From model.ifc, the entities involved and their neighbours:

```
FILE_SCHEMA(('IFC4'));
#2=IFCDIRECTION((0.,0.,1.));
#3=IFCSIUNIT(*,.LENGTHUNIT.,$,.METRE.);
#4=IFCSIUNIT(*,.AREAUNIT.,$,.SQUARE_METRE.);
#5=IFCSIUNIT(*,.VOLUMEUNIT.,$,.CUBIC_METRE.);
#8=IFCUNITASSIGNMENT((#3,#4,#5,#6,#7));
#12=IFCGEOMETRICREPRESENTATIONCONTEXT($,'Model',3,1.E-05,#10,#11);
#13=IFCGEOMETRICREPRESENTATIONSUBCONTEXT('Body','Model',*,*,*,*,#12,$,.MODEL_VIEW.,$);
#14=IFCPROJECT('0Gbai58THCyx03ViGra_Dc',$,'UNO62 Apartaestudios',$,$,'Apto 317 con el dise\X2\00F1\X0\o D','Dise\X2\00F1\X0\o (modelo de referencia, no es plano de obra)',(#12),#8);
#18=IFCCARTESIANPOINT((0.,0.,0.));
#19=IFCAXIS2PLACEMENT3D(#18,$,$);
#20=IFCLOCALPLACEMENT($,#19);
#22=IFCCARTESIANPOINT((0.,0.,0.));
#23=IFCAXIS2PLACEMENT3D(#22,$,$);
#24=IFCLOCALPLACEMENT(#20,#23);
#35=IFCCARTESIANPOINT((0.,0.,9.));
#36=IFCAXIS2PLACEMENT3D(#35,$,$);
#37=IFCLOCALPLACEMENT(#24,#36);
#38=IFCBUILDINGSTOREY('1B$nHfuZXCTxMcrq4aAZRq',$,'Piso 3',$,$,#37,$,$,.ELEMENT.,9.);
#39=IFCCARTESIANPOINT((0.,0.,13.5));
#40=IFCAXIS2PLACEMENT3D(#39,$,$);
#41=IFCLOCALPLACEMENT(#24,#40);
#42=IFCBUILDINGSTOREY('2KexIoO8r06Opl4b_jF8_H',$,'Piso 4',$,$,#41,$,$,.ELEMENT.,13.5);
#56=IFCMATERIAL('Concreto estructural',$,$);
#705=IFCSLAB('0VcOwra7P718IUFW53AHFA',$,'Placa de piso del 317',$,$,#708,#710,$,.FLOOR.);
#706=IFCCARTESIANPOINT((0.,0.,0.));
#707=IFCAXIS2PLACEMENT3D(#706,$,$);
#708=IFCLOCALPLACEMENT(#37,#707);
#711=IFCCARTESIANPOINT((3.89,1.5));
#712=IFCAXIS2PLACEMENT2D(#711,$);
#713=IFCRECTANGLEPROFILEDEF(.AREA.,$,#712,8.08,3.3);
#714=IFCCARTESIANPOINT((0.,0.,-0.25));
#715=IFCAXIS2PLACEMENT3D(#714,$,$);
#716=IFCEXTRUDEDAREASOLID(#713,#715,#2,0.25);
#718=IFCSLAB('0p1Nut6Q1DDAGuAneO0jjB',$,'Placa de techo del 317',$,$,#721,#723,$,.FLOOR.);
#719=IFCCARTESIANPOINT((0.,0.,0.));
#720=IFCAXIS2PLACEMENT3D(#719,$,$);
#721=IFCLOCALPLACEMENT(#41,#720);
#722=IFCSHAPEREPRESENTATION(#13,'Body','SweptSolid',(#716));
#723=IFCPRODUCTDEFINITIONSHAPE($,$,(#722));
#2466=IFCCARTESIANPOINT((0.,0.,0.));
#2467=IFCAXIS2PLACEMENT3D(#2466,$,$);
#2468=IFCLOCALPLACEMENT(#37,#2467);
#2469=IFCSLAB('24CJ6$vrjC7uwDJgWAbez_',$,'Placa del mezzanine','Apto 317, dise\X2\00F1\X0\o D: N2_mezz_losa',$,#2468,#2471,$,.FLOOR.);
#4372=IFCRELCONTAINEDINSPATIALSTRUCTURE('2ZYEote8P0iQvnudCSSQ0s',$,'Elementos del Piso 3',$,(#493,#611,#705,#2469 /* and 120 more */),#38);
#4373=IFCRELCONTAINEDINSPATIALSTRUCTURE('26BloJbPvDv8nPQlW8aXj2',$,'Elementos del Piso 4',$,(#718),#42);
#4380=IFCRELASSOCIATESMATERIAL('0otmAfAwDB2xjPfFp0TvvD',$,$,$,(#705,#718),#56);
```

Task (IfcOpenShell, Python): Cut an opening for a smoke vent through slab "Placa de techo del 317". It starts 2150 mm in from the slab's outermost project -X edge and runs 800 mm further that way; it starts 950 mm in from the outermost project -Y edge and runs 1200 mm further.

```python
import numpy as np
import ifcopenshell
import ifcopenshell.api.feature
import ifcopenshell.api.geometry
import ifcopenshell.api.root
import ifcopenshell.geom
import ifcopenshell.util.placement
import ifcopenshell.util.representation
import ifcopenshell.util.shape
import ifcopenshell.util.unit

model = ifcopenshell.open("model.ifc")
unit_scale = ifcopenshell.util.unit.calculate_unit_scale(model)
settings = ifcopenshell.geom.settings()


def volume(element):
    """Net volume in cubic metres, openings subtracted."""
    shape = ifcopenshell.geom.create_shape(settings, element)
    return ifcopenshell.util.shape.get_volume(shape.geometry)


slab = model.by_guid("0p1Nut6Q1DDAGuAneO0jjB")
before = volume(slab)

# Extent in the slab's own axes, in metres. The edges named are its -X and -Y sides.
slab_shape = ifcopenshell.geom.create_shape(settings, slab)
vertices = ifcopenshell.util.shape.get_vertices(slab_shape.geometry)
x_min, y_min, bottom = vertices.min(axis=0)
top = vertices[:, 2].max()

opening = ifcopenshell.api.root.create_entity(model, ifc_class="IfcOpeningElement", name="Smoke vent opening", predefined_type="OPENING")
context = ifcopenshell.util.representation.get_context(model, "Model", "Body", "MODEL_VIEW")
width, depth = 0.8, 1.2
outline = [(0.0, 0.0), (width, 0.0), (width, depth), (0.0, depth), (0.0, 0.0)]
# Overshoot both faces by 50 mm so the cut is clean.
shape = ifcopenshell.api.geometry.add_slab_representation(
    model, context=context, depth=top - bottom + 0.1, polyline=outline
)
ifcopenshell.api.geometry.assign_representation(model, product=opening, representation=shape)

matrix = ifcopenshell.util.placement.get_local_placement(slab.ObjectPlacement)
matrix[:, 3] = matrix @ np.append(np.array([x_min + 2.15, y_min + 0.95, bottom - 0.05]) / unit_scale, 1.0)
ifcopenshell.api.geometry.edit_object_placement(model, product=opening, matrix=matrix, is_si=False)
ifcopenshell.api.feature.add_feature(model, feature=opening, element=slab)

after = volume(slab)

print(f"slab volume {before:.3f} -> {after:.3f} m3")

model.write("model_v2.ifc")
```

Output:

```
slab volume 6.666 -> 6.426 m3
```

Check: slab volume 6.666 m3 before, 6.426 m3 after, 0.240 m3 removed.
